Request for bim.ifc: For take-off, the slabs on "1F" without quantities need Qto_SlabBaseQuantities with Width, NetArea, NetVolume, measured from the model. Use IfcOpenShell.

First a look at what the model holds.

```python
import ifcopenshell
import ifcopenshell.util.element
import ifcopenshell.util.unit

model = ifcopenshell.open("bim.ifc")
print(model.schema)
for unit_type in ("LENGTHUNIT", "AREAUNIT", "VOLUMEUNIT"):
    print(unit_type, ifcopenshell.util.unit.calculate_unit_scale(model, unit_type))
storey = next(s for s in model.by_type("IfcBuildingStorey") if s.Name == "1F")
slabs = [e for e in ifcopenshell.util.element.get_decomposition(storey) if e.is_a("IfcSlab")]
for e in sorted(slabs, key=lambda e: e.id()):
    print(e.id(), e.is_a(), e.Name, list(ifcopenshell.util.element.get_psets(e, qtos_only=True)), sep=" | ")
```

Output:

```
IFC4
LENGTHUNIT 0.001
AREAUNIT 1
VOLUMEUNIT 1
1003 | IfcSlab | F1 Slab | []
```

```python
import ifcopenshell
import ifcopenshell.api.pset
import ifcopenshell.geom
import ifcopenshell.util.element
import ifcopenshell.util.shape
import ifcopenshell.util.unit

model = ifcopenshell.open("bim.ifc")
unit_scale = ifcopenshell.util.unit.calculate_unit_scale(model)
area_scale = ifcopenshell.util.unit.calculate_unit_scale(model, "AREAUNIT")
volume_scale = ifcopenshell.util.unit.calculate_unit_scale(model, "VOLUMEUNIT")
settings = ifcopenshell.geom.settings()

storey = next(s for s in model.by_type("IfcBuildingStorey") if s.Name == "1F")
slabs = [e for e in ifcopenshell.util.element.get_decomposition(storey) if e.is_a("IfcSlab")]

for e in sorted(slabs, key=lambda e: e.id()):
    if ifcopenshell.util.element.get_psets(e, qtos_only=True, should_inherit=False):
        continue
    # Geometry comes back in metres, in the element's own axes.
    shape = ifcopenshell.geom.create_shape(settings, e)
    values = {
        "Width": ifcopenshell.util.shape.get_z(shape.geometry) / unit_scale,
        "NetArea": ifcopenshell.util.shape.get_footprint_area(shape.geometry) / area_scale,
        "NetVolume": ifcopenshell.util.shape.get_volume(shape.geometry) / volume_scale,
    }
    qto = ifcopenshell.api.pset.add_qto(model, product=e, name="Qto_SlabBaseQuantities")
    ifcopenshell.api.pset.edit_qto(model, qto=qto, properties=values)
    print(e.id(), {k: round(v, 3) for k, v in values.items()})

model.write("bim-out.ifc")
```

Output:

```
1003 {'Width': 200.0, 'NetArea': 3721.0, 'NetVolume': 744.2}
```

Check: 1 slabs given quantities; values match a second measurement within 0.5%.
